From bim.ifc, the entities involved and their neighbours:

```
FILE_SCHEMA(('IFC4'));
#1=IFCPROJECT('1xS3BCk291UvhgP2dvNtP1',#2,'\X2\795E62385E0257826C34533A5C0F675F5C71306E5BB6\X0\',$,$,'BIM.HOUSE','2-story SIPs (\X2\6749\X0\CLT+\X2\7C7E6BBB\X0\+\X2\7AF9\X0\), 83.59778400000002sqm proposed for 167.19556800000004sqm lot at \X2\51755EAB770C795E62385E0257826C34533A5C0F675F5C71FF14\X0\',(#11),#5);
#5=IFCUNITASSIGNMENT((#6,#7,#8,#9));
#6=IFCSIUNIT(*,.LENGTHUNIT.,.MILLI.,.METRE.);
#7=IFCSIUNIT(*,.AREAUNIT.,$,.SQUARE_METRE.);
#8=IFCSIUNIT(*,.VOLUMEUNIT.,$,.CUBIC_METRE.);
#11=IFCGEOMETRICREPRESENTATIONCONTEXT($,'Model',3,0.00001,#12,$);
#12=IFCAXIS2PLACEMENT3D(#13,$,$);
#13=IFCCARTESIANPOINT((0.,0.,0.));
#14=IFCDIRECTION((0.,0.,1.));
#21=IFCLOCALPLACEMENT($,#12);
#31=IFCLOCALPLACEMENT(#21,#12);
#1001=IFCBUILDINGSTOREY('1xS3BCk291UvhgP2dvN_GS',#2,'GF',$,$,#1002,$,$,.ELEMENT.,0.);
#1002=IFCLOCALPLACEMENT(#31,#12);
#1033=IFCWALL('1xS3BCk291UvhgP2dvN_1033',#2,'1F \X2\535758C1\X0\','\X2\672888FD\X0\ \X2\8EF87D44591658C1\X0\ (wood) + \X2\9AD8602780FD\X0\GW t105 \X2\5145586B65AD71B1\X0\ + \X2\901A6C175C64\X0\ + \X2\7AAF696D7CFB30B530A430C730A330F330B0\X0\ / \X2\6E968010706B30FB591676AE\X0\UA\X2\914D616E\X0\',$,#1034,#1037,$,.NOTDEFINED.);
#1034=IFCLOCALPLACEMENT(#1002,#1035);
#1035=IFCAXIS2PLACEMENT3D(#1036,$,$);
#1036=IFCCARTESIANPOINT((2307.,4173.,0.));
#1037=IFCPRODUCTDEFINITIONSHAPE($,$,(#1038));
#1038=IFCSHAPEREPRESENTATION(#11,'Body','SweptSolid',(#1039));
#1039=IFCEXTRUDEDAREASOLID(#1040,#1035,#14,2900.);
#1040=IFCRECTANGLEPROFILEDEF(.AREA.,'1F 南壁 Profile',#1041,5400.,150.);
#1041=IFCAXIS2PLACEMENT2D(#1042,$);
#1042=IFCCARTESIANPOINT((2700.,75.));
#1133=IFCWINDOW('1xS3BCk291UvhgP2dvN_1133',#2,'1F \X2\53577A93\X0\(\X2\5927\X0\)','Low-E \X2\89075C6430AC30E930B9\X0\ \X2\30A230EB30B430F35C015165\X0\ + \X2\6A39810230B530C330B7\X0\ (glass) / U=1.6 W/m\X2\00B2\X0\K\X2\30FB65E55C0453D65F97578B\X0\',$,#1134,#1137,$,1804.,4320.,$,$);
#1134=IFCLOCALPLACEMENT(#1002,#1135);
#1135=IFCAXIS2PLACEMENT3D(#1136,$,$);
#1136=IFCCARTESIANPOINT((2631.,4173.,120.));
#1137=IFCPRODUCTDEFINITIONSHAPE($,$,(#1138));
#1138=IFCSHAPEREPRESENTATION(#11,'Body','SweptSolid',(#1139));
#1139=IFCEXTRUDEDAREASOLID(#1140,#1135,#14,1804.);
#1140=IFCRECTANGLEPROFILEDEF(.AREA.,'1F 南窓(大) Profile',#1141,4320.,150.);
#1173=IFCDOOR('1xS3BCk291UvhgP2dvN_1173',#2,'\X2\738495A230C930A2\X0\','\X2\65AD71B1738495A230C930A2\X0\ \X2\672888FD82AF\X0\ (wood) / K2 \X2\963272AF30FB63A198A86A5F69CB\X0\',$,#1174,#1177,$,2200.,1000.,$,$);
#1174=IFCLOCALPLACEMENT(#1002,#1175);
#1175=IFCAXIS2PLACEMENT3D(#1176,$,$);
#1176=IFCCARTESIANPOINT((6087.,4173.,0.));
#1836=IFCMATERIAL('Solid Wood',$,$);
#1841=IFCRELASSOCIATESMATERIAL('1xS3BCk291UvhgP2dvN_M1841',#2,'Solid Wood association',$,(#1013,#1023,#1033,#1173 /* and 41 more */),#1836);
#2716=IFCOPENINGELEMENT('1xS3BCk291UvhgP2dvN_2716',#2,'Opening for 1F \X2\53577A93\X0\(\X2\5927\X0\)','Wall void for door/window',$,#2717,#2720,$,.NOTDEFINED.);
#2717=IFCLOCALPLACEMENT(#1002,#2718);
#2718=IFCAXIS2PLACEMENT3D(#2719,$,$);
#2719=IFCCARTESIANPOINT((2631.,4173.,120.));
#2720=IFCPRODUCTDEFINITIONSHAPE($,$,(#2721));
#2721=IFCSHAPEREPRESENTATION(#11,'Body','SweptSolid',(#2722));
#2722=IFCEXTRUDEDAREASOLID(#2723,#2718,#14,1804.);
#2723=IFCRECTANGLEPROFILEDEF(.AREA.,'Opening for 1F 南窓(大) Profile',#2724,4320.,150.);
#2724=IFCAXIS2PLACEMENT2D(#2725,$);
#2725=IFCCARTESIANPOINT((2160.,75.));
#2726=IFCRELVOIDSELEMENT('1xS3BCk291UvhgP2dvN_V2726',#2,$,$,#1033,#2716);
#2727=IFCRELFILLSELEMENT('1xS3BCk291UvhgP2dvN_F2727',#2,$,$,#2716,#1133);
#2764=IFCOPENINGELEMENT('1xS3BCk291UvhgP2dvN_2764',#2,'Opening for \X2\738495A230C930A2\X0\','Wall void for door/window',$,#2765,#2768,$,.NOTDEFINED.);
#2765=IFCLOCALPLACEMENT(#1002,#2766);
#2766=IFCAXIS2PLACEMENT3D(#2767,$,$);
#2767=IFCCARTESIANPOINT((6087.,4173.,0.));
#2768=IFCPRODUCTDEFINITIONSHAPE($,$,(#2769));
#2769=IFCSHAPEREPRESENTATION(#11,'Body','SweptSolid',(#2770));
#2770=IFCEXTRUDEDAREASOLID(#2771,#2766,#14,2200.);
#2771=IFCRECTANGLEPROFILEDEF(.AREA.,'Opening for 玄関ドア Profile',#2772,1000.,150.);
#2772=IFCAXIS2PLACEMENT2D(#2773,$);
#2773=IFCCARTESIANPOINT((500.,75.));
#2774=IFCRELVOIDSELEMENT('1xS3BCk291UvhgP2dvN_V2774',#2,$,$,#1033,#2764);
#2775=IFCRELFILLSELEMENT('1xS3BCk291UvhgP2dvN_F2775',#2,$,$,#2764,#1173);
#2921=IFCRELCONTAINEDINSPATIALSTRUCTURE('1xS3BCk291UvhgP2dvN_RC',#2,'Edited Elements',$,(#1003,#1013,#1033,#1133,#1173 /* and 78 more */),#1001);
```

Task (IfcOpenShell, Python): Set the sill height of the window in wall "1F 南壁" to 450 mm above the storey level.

```python
import numpy as np
import ifcopenshell
import ifcopenshell.api.geometry
import ifcopenshell.geom
import ifcopenshell.util.element
import ifcopenshell.util.placement
import ifcopenshell.util.shape
import ifcopenshell.util.unit

model = ifcopenshell.open("bim.ifc")
unit_scale = ifcopenshell.util.unit.calculate_unit_scale(model)

window = model.by_guid("1xS3BCk291UvhgP2dvN_1133")
opening = window.FillsVoids[0].RelatingOpeningElement
storey = ifcopenshell.util.element.get_container(window, ifc_class="IfcBuildingStorey")
level = ifcopenshell.util.placement.get_local_placement(storey.ObjectPlacement)[2, 3]

# The opening's origin need not be at the sill, so measure its lowest point.
shape = ifcopenshell.geom.create_shape(ifcopenshell.geom.settings(), opening)
bottom = ifcopenshell.util.shape.get_shape_bottom_elevation(shape, shape.geometry) / unit_scale
dz = level + 450.0 - bottom

shift = np.array([0.0, 0.0, dz])
# The window is not placed relative to its opening, so move both.
for product in (opening, window):
    matrix = ifcopenshell.util.placement.get_local_placement(product.ObjectPlacement)
    matrix[:3, 3] += shift
    ifcopenshell.api.geometry.edit_object_placement(model, product=product, matrix=matrix, is_si=False)

print(f"moved by {dz * unit_scale:+.3f} m")

model.write("bim_v2.ifc")
```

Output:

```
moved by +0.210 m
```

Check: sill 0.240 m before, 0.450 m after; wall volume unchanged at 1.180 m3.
